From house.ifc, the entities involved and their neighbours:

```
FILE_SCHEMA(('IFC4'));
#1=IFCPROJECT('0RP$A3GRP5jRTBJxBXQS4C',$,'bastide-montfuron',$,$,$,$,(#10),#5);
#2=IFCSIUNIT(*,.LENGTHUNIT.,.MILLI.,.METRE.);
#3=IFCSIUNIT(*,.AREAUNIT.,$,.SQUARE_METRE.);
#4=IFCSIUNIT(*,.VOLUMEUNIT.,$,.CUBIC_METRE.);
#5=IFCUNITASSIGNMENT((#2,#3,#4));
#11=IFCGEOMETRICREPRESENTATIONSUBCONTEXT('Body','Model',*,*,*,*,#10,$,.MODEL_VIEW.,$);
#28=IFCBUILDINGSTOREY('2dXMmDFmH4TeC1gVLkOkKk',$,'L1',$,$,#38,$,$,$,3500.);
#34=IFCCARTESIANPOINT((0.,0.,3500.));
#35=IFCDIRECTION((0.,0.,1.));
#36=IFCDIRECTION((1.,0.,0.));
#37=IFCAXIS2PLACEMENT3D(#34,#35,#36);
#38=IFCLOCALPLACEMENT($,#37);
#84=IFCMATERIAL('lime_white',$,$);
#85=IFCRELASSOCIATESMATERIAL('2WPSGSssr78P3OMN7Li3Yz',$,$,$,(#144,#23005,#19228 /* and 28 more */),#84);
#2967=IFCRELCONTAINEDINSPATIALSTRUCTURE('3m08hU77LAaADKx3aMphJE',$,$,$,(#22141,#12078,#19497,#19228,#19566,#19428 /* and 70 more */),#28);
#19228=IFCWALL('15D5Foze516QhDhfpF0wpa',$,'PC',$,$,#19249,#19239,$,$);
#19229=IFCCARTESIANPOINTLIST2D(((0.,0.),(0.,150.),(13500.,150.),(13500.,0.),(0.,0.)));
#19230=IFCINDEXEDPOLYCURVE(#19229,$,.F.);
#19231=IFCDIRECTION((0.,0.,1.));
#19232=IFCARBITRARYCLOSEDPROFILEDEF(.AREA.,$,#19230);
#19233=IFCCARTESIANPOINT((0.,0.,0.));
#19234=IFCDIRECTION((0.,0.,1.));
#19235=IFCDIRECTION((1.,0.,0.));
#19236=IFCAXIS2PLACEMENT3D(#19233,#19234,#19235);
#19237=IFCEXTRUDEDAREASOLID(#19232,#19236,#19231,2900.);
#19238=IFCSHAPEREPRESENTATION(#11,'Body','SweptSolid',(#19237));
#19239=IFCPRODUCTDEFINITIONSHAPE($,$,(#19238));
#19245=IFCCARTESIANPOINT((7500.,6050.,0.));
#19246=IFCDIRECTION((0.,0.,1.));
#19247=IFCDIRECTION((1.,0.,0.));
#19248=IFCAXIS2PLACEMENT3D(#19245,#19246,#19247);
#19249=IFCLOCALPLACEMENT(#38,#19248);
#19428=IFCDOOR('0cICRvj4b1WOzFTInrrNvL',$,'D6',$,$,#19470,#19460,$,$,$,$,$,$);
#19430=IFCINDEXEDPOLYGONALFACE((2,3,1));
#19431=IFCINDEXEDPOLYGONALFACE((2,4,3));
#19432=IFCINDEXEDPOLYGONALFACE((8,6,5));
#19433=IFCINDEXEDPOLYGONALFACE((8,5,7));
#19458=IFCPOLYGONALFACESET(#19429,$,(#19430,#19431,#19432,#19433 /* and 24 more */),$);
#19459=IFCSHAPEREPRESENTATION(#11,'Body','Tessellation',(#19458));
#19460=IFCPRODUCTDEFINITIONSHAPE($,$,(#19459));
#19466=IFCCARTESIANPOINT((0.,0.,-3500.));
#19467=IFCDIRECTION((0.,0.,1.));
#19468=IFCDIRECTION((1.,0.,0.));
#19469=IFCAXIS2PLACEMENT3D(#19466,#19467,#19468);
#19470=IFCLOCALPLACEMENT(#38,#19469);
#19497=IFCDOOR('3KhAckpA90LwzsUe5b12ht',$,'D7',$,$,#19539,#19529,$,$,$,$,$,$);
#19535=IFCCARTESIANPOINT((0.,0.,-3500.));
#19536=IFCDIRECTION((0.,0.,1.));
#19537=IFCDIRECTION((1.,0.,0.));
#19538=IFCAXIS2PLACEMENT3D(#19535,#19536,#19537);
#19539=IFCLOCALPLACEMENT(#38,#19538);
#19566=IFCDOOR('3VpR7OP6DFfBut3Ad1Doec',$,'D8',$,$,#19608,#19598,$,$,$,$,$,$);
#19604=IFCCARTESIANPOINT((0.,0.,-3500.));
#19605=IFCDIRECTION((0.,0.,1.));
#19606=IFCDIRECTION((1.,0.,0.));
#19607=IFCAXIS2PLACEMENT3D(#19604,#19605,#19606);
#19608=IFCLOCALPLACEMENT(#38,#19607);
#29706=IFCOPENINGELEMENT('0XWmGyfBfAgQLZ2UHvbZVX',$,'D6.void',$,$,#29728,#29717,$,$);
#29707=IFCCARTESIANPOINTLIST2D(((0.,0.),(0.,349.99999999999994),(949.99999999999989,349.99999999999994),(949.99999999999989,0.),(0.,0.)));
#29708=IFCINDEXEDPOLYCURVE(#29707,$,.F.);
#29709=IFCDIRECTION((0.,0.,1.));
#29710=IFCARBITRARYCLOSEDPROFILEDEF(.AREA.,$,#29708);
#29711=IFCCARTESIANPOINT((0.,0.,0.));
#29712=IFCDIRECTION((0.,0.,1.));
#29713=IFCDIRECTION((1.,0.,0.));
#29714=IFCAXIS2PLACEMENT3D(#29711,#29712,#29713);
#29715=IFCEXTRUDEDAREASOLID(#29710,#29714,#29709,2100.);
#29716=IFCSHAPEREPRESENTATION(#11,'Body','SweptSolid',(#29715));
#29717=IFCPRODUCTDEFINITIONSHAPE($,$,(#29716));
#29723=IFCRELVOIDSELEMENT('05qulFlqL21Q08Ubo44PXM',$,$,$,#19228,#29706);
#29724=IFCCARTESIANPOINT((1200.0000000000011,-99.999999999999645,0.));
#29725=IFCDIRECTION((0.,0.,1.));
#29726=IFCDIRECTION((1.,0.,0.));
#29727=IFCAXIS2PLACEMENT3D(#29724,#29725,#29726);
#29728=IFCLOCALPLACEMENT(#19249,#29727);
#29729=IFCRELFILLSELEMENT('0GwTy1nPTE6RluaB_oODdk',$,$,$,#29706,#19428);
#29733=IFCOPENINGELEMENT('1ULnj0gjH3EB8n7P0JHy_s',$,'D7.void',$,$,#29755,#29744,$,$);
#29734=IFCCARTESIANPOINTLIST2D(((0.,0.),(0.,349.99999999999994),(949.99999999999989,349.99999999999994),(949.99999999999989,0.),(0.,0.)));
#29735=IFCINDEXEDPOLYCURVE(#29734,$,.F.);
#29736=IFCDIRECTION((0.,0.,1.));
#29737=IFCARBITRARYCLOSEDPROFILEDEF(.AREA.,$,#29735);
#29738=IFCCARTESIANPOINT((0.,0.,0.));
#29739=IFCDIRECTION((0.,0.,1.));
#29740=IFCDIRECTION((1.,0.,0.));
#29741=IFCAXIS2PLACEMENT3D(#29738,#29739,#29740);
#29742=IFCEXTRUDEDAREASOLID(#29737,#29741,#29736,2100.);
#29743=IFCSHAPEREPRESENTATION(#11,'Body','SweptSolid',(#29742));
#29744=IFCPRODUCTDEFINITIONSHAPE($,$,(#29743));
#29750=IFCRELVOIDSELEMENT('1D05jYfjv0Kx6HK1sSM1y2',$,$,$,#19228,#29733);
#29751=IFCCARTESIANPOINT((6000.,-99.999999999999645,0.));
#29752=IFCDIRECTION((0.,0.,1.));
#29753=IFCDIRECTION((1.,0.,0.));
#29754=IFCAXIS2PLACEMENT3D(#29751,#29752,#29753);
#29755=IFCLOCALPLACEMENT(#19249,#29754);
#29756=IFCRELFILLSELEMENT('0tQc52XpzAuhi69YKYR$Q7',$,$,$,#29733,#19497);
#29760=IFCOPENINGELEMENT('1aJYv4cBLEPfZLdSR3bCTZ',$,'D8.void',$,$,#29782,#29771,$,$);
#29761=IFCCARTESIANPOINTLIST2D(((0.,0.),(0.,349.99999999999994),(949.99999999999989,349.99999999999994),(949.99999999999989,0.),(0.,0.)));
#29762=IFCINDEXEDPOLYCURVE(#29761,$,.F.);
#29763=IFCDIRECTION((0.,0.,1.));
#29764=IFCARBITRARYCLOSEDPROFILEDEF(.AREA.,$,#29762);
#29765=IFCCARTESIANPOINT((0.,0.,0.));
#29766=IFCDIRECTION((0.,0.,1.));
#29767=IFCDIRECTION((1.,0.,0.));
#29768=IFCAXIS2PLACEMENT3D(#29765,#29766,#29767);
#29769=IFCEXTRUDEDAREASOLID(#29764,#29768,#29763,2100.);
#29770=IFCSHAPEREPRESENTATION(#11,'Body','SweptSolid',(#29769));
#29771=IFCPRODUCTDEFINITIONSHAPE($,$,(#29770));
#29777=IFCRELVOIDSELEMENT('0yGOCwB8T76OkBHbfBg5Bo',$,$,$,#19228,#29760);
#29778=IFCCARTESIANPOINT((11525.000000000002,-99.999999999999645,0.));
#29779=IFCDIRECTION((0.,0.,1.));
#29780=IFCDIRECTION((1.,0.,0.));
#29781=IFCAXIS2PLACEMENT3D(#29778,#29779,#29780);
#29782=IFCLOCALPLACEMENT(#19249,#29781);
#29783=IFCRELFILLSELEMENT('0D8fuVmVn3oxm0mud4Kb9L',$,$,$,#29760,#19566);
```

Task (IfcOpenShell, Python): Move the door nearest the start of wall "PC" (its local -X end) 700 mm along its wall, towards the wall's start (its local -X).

```python
import ifcopenshell
import ifcopenshell.api.geometry
import ifcopenshell.util.placement
import ifcopenshell.util.unit

model = ifcopenshell.open("house.ifc")
unit_scale = ifcopenshell.util.unit.calculate_unit_scale(model)

door = model.by_guid("0cICRvj4b1WOzFTInrrNvL")
opening = door.FillsVoids[0].RelatingOpeningElement
wall = opening.VoidsElements[0].RelatingBuildingElement

wall_matrix = ifcopenshell.util.placement.get_local_placement(wall.ObjectPlacement)
shift = wall_matrix[:3, 0] * -0.7 / unit_scale
before = ifcopenshell.util.placement.get_local_placement(door.ObjectPlacement)[:3, 3].copy()

# The door is not placed relative to its opening, so move both.
for product in (opening, door):
    matrix = ifcopenshell.util.placement.get_local_placement(product.ObjectPlacement)
    matrix[:3, 3] += shift
    ifcopenshell.api.geometry.edit_object_placement(model, product=product, matrix=matrix, is_si=False)

after = ifcopenshell.util.placement.get_local_placement(door.ObjectPlacement)[:3, 3]
print("door moved by", (after - before).round(3) + 0.0)

model.write("house_edited.ifc")
```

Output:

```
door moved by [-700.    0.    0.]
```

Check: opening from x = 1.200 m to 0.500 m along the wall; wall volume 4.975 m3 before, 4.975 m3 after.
